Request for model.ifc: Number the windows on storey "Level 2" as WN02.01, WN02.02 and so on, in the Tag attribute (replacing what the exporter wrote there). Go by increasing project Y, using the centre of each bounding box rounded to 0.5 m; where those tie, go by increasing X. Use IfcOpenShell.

First a look at what the model holds.

```python
import ifcopenshell
import ifcopenshell.util.element
import ifcopenshell.util.placement

model = ifcopenshell.open("model.ifc")
print(model.schema)
storey = next(s for s in model.by_type("IfcBuildingStorey") if s.Name == "Level 2")
windows = [e for e in ifcopenshell.util.element.get_decomposition(storey) if e.is_a("IfcWindow")]
for e in sorted(windows, key=lambda e: e.id()):
    origin = ifcopenshell.util.placement.get_local_placement(e.ObjectPlacement)[:3, 3]
    print(e.id(), e.Tag, e.Name, origin.round(2) + 0.0, sep=" | ")
```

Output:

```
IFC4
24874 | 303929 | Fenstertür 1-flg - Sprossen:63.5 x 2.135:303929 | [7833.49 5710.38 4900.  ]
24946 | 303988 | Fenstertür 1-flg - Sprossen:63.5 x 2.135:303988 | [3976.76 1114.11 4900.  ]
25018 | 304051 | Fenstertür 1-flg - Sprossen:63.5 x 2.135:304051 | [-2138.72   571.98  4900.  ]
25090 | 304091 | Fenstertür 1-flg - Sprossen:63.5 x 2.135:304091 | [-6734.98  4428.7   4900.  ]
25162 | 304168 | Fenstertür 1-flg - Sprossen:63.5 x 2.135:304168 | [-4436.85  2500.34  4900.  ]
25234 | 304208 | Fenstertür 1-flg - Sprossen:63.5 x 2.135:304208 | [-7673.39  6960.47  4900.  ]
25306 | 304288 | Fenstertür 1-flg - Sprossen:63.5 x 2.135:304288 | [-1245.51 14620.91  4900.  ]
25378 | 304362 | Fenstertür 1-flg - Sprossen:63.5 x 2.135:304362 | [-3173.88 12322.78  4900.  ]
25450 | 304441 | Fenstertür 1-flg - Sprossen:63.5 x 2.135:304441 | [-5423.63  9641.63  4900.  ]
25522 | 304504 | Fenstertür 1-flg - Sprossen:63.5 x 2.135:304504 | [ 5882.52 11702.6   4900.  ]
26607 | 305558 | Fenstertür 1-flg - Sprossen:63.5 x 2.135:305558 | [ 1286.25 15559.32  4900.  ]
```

```python
import ifcopenshell
import ifcopenshell.geom
import ifcopenshell.util.element
import ifcopenshell.util.shape

model = ifcopenshell.open("model.ifc")
settings = ifcopenshell.geom.settings()
settings.set("use-world-coords", True)


def centre(element):
    shape = ifcopenshell.geom.create_shape(settings, element)
    return ifcopenshell.util.shape.get_bbox_centroid(shape.geometry)


storey = next(s for s in model.by_type("IfcBuildingStorey") if s.Name == "Level 2")
windows = [e for e in ifcopenshell.util.element.get_decomposition(storey) if e.is_a("IfcWindow")]

# Insertion points can sit at a corner or the storey origin, so sort by the geometry (in metres).
centres = {e: centre(e) for e in windows}
windows.sort(key=lambda e: (round(centres[e][1] / 0.5), centres[e][0]))

for i, e in enumerate(windows, start=1):
    number = f"WN02.{i:02d}"
    e.Tag = number
    print(e.id(), number)

model.write("model_rev.ifc")
```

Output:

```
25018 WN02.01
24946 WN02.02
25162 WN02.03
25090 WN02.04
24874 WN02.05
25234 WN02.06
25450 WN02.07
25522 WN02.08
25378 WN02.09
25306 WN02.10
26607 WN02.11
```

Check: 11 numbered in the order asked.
